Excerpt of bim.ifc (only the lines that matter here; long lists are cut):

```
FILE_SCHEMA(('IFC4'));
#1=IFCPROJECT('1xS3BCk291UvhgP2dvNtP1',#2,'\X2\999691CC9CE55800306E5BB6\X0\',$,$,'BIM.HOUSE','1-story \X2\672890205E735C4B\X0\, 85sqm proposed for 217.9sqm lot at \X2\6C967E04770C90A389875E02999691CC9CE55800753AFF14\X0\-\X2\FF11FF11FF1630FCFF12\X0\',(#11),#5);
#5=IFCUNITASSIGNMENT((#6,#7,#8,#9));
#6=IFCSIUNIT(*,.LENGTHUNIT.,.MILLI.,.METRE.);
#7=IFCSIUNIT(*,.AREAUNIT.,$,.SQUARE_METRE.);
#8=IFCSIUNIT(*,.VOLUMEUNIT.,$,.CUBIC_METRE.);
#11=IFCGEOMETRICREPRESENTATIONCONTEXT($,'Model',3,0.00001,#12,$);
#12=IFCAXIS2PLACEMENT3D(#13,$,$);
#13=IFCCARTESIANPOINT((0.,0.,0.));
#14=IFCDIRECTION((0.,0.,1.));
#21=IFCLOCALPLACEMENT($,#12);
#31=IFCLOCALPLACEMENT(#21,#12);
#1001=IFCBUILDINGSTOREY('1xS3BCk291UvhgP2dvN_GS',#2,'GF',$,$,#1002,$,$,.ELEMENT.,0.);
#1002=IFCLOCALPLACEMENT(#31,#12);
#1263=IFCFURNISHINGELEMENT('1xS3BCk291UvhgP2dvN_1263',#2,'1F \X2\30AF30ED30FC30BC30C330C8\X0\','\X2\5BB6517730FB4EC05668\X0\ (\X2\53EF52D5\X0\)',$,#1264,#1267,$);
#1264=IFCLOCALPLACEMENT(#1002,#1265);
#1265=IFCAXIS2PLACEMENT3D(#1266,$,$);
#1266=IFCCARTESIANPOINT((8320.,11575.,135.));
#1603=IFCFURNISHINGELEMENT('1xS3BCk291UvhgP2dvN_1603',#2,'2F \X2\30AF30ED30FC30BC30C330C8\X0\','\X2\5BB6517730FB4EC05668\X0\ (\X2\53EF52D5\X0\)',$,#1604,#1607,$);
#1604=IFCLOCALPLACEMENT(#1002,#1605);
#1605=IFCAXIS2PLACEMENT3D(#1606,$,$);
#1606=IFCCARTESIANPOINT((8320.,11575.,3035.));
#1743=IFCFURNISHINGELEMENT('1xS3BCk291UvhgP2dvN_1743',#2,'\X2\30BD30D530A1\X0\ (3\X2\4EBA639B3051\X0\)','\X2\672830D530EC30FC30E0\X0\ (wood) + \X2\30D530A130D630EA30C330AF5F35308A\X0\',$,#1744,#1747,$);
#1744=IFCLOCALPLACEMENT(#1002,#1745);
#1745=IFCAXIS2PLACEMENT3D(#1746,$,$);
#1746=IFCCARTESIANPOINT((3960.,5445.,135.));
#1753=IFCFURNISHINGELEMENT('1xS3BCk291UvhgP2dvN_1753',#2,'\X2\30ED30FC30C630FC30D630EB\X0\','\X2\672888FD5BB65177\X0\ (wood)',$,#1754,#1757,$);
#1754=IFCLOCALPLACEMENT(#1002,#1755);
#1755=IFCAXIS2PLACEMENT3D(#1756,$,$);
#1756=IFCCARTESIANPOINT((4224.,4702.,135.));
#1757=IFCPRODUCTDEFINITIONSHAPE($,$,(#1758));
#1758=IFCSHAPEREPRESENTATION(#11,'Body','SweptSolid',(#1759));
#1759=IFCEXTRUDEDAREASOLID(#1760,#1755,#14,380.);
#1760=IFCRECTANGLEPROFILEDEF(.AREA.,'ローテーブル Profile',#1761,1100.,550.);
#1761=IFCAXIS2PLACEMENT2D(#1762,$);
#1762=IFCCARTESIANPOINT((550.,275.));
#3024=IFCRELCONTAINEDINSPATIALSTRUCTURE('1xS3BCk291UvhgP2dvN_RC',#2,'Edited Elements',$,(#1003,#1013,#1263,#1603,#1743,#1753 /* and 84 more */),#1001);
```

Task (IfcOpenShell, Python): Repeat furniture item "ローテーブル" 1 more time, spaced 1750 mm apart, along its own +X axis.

```python
import ifcopenshell
import ifcopenshell.api.geometry
import ifcopenshell.api.root
import ifcopenshell.util.element
import ifcopenshell.util.placement
import ifcopenshell.util.unit

model = ifcopenshell.open("bim.ifc")
unit_scale = ifcopenshell.util.unit.calculate_unit_scale(model)


def reuse_history(source, copy):
    """copy_class also copies each property set's owner history, people and application; keep the originals."""
    for rel in copy.IsDefinedBy:
        if rel.is_a("IfcRelDefinesByProperties") and (history := rel.RelatingPropertyDefinition.OwnerHistory):
            rel.RelatingPropertyDefinition.OwnerHistory = source.OwnerHistory
            ifcopenshell.util.element.remove_deep2(model, history)


source = model.by_guid("1xS3BCk291UvhgP2dvN_1753")
base = ifcopenshell.util.placement.get_local_placement(source.ObjectPlacement)
step = base[:3, 0] * 1.75 / unit_scale

for i in range(1, 2):
    copy = ifcopenshell.api.root.copy_class(model, product=source)
    copy.Representation = ifcopenshell.util.element.copy_deep(
        model, source.Representation, exclude=["IfcGeometricRepresentationContext", "IfcRepresentationMap"]
    )
    reuse_history(source, copy)
    matrix = base.copy()
    matrix[:3, 3] += i * step
    print("added at", matrix[:3, 3].round(3) + 0.0)
    ifcopenshell.api.geometry.edit_object_placement(model, product=copy, matrix=matrix, is_si=False)

model.write("bim_edited.ifc")
```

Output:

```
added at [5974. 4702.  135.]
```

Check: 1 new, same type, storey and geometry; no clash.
